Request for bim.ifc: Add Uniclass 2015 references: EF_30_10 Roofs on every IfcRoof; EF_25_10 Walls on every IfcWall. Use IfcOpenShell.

First a look at what the model holds.

```python
import ifcopenshell

model = ifcopenshell.open("bim.ifc")
print(model.schema)
print("classifications:", [c.Name for c in model.by_type("IfcClassification")])
for ifc_class in ("IfcDoor", "IfcRoof", "IfcStair", "IfcWall", "IfcWindow"):
    print(ifc_class, len(model.by_type(ifc_class)))
```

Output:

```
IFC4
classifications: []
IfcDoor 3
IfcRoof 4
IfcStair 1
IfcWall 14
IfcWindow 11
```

```python
import ifcopenshell
import ifcopenshell.api.classification

model = ifcopenshell.open("bim.ifc")

system = ifcopenshell.api.classification.add_classification(model, classification="Uniclass 2015")

codes = {
    "IfcRoof": ("EF_30_10", "Roofs"),
    "IfcWall": ("EF_25_10", "Walls"),
}
for ifc_class, (code, name) in codes.items():
    products = model.by_type(ifc_class)
    ifcopenshell.api.classification.add_reference(
        model, products=products, classification=system, identification=code, name=name
    )
    print(code, len(products))

model.write("bim_edited.ifc")
```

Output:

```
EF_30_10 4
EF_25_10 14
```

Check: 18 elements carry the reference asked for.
